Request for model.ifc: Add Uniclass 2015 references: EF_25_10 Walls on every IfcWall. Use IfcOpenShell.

First a look at what the model holds.

```python
import ifcopenshell

model = ifcopenshell.open("model.ifc")
print(model.schema)
print("classifications:", [c.Name for c in model.by_type("IfcClassification")])
for ifc_class in ("IfcDoor", "IfcRoof", "IfcStair", "IfcWall", "IfcWindow"):
    print(ifc_class, len(model.by_type(ifc_class)))
```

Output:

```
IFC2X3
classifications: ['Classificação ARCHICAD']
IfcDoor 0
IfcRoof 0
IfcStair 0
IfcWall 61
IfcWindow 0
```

```python
import ifcopenshell
import ifcopenshell.api.classification

model = ifcopenshell.open("model.ifc")

# IFC2X3 requires Source and Edition and has no link from the project to the system.
system = model.create_entity("IfcClassification", Source="NBS", Edition="2015", Name="Uniclass 2015")

codes = {
    "IfcWall": ("EF_25_10", "Walls"),
}
for ifc_class, (code, name) in codes.items():
    products = model.by_type(ifc_class)
    ifcopenshell.api.classification.add_reference(
        model, products=products, classification=system, identification=code, name=name
    )
    print(code, len(products))

model.write("model-out.ifc")
```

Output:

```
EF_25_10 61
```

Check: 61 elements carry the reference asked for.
